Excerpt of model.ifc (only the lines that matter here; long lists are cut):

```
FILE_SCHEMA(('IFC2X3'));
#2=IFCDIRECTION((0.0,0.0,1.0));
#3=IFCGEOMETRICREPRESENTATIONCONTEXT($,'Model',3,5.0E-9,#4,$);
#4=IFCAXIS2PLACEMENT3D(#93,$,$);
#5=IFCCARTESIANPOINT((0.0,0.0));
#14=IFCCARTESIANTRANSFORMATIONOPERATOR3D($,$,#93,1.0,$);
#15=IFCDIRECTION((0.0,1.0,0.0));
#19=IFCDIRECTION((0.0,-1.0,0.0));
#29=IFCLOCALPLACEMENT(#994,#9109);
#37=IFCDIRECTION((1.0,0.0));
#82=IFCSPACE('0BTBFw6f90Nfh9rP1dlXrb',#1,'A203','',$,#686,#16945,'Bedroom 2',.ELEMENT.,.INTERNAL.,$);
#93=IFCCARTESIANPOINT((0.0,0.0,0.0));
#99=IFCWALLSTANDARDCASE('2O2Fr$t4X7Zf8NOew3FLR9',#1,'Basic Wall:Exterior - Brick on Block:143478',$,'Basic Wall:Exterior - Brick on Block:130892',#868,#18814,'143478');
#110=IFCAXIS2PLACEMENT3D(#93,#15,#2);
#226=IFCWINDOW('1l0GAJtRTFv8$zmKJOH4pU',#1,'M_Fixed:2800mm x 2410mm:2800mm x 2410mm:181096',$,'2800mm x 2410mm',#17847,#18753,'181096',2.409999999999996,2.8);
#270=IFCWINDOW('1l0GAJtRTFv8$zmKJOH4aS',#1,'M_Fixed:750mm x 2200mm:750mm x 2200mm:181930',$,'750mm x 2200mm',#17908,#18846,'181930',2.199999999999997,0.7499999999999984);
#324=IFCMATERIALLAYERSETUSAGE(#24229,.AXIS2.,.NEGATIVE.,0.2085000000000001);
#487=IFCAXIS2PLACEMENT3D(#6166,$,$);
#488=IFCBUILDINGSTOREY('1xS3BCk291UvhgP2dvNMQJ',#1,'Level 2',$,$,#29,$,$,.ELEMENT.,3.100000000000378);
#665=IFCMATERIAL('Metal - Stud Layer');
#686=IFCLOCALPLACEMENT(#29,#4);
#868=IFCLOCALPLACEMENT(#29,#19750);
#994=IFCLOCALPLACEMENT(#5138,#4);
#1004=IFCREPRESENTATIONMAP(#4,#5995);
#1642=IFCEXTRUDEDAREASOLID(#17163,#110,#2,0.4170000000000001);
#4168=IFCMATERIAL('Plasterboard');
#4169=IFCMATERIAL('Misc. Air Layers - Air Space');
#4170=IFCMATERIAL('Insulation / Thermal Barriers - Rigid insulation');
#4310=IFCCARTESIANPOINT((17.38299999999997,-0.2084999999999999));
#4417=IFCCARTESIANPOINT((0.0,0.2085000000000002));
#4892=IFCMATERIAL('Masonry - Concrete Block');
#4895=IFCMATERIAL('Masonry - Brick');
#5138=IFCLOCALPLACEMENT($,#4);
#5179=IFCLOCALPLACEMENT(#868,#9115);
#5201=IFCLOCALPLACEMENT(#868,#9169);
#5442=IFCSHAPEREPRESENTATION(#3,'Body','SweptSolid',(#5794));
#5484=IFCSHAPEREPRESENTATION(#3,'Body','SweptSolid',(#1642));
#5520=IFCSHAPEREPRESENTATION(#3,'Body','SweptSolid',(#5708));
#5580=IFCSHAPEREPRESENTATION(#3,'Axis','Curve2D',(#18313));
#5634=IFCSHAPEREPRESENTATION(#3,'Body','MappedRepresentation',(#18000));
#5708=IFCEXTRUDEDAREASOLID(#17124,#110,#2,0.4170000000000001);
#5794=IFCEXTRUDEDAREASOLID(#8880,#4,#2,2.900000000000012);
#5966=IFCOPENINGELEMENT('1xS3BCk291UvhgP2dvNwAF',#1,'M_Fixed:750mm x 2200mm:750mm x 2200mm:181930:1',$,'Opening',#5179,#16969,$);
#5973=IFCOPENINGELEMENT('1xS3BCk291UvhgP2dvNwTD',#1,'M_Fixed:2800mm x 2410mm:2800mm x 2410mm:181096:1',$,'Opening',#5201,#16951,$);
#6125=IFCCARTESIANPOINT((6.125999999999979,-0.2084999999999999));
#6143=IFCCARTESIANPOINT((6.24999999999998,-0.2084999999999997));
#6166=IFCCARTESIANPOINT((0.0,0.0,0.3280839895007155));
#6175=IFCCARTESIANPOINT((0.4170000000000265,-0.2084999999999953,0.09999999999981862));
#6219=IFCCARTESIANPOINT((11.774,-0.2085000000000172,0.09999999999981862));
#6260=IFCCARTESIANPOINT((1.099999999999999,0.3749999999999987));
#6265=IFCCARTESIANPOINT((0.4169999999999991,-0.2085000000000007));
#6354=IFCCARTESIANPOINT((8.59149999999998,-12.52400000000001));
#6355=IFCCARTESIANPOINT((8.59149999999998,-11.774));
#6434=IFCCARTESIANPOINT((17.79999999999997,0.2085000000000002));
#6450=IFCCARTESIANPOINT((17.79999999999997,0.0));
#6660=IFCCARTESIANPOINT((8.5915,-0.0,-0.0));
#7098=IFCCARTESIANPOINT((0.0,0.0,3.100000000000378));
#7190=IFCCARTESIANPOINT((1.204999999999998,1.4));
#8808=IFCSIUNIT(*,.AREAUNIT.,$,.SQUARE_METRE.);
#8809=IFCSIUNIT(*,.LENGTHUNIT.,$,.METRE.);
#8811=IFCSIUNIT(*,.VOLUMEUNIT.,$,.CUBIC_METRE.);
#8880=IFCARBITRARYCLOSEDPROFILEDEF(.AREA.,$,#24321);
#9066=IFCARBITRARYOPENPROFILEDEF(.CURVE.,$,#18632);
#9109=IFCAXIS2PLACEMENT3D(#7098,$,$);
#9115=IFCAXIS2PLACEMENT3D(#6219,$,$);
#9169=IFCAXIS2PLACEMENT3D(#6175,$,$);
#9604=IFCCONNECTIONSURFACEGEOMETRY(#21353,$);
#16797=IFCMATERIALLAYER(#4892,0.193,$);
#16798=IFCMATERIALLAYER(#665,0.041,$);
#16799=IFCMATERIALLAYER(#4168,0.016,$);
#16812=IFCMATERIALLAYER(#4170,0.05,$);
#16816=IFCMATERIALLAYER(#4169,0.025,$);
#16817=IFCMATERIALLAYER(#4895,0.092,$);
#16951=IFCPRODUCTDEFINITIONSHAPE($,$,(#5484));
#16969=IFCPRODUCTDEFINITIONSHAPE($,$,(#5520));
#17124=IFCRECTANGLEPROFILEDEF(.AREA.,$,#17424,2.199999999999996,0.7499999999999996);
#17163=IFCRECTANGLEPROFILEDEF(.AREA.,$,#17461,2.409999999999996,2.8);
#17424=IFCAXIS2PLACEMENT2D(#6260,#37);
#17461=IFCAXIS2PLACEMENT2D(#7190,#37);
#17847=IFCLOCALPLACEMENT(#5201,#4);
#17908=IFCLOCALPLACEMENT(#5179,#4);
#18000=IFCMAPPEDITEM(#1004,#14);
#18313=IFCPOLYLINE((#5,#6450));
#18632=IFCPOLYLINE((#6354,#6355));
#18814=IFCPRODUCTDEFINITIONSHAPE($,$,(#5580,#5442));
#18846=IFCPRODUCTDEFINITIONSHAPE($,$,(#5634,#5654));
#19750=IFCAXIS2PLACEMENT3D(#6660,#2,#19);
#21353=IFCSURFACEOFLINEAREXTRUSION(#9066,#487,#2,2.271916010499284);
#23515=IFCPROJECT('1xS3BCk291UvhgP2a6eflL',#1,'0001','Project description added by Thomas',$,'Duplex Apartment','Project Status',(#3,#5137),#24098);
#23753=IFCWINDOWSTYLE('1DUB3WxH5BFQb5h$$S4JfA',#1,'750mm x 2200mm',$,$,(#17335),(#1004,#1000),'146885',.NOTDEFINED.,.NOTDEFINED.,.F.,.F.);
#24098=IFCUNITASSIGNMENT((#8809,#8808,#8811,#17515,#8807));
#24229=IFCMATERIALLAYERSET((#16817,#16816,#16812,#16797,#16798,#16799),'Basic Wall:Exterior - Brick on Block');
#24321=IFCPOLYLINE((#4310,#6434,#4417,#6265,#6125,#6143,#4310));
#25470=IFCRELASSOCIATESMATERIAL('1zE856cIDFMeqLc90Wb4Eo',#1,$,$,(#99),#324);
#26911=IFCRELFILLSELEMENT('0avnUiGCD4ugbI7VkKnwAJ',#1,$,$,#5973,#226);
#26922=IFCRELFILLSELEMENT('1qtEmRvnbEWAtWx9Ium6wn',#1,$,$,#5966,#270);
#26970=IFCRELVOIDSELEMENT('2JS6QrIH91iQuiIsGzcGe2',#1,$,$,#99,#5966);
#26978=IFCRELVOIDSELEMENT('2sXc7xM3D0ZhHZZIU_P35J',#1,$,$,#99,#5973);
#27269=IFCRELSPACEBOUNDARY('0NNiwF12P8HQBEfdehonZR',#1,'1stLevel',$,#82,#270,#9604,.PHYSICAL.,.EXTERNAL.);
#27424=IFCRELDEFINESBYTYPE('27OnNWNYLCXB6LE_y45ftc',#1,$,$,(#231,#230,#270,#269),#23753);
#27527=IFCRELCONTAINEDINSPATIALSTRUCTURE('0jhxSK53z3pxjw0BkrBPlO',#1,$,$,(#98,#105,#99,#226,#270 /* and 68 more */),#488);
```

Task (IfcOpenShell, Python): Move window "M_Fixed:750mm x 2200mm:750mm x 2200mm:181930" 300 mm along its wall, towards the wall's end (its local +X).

```python
import numpy as np
import ifcopenshell
import ifcopenshell.api.geometry
import ifcopenshell.util.placement
import ifcopenshell.util.unit

model = ifcopenshell.open("model.ifc")
unit_scale = ifcopenshell.util.unit.calculate_unit_scale(model)

window = model.by_guid("1l0GAJtRTFv8$zmKJOH4aS")
opening = window.FillsVoids[0].RelatingOpeningElement
wall = opening.VoidsElements[0].RelatingBuildingElement

wall_matrix = ifcopenshell.util.placement.get_local_placement(wall.ObjectPlacement)
shift = wall_matrix[:3, 0] * 0.3 / unit_scale
before = ifcopenshell.util.placement.get_local_placement(window.ObjectPlacement)[:3, 3].copy()

# The window is placed relative to its opening, so it follows when the opening moves.
matrix = ifcopenshell.util.placement.get_local_placement(opening.ObjectPlacement)
matrix[:3, 3] += shift
ifcopenshell.api.geometry.edit_object_placement(
    model, product=opening, matrix=matrix, is_si=False, should_transform_children=True
)

# Space boundary surfaces are stored in each space's coordinates; move them too.
for rel in window.ProvidesBoundaries:
    if not rel.ConnectionGeometry:
        continue
    surface = rel.ConnectionGeometry.SurfaceOnRelatingElement
    space_matrix = ifcopenshell.util.placement.get_local_placement(rel.RelatingSpace.ObjectPlacement)
    point = np.array(surface.Position.Location.Coordinates) + space_matrix[:3, :3].T @ shift
    surface.Position = model.createIfcAxis2Placement3D(
        model.createIfcCartesianPoint(point.tolist()), surface.Position.Axis, surface.Position.RefDirection
    )

after = ifcopenshell.util.placement.get_local_placement(window.ObjectPlacement)[:3, 3]
print("window moved by", (after - before).round(3) + 0.0)

model.write("model_edited.ifc")
```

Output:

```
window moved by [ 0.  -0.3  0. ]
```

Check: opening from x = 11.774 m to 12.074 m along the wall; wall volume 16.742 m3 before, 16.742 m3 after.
